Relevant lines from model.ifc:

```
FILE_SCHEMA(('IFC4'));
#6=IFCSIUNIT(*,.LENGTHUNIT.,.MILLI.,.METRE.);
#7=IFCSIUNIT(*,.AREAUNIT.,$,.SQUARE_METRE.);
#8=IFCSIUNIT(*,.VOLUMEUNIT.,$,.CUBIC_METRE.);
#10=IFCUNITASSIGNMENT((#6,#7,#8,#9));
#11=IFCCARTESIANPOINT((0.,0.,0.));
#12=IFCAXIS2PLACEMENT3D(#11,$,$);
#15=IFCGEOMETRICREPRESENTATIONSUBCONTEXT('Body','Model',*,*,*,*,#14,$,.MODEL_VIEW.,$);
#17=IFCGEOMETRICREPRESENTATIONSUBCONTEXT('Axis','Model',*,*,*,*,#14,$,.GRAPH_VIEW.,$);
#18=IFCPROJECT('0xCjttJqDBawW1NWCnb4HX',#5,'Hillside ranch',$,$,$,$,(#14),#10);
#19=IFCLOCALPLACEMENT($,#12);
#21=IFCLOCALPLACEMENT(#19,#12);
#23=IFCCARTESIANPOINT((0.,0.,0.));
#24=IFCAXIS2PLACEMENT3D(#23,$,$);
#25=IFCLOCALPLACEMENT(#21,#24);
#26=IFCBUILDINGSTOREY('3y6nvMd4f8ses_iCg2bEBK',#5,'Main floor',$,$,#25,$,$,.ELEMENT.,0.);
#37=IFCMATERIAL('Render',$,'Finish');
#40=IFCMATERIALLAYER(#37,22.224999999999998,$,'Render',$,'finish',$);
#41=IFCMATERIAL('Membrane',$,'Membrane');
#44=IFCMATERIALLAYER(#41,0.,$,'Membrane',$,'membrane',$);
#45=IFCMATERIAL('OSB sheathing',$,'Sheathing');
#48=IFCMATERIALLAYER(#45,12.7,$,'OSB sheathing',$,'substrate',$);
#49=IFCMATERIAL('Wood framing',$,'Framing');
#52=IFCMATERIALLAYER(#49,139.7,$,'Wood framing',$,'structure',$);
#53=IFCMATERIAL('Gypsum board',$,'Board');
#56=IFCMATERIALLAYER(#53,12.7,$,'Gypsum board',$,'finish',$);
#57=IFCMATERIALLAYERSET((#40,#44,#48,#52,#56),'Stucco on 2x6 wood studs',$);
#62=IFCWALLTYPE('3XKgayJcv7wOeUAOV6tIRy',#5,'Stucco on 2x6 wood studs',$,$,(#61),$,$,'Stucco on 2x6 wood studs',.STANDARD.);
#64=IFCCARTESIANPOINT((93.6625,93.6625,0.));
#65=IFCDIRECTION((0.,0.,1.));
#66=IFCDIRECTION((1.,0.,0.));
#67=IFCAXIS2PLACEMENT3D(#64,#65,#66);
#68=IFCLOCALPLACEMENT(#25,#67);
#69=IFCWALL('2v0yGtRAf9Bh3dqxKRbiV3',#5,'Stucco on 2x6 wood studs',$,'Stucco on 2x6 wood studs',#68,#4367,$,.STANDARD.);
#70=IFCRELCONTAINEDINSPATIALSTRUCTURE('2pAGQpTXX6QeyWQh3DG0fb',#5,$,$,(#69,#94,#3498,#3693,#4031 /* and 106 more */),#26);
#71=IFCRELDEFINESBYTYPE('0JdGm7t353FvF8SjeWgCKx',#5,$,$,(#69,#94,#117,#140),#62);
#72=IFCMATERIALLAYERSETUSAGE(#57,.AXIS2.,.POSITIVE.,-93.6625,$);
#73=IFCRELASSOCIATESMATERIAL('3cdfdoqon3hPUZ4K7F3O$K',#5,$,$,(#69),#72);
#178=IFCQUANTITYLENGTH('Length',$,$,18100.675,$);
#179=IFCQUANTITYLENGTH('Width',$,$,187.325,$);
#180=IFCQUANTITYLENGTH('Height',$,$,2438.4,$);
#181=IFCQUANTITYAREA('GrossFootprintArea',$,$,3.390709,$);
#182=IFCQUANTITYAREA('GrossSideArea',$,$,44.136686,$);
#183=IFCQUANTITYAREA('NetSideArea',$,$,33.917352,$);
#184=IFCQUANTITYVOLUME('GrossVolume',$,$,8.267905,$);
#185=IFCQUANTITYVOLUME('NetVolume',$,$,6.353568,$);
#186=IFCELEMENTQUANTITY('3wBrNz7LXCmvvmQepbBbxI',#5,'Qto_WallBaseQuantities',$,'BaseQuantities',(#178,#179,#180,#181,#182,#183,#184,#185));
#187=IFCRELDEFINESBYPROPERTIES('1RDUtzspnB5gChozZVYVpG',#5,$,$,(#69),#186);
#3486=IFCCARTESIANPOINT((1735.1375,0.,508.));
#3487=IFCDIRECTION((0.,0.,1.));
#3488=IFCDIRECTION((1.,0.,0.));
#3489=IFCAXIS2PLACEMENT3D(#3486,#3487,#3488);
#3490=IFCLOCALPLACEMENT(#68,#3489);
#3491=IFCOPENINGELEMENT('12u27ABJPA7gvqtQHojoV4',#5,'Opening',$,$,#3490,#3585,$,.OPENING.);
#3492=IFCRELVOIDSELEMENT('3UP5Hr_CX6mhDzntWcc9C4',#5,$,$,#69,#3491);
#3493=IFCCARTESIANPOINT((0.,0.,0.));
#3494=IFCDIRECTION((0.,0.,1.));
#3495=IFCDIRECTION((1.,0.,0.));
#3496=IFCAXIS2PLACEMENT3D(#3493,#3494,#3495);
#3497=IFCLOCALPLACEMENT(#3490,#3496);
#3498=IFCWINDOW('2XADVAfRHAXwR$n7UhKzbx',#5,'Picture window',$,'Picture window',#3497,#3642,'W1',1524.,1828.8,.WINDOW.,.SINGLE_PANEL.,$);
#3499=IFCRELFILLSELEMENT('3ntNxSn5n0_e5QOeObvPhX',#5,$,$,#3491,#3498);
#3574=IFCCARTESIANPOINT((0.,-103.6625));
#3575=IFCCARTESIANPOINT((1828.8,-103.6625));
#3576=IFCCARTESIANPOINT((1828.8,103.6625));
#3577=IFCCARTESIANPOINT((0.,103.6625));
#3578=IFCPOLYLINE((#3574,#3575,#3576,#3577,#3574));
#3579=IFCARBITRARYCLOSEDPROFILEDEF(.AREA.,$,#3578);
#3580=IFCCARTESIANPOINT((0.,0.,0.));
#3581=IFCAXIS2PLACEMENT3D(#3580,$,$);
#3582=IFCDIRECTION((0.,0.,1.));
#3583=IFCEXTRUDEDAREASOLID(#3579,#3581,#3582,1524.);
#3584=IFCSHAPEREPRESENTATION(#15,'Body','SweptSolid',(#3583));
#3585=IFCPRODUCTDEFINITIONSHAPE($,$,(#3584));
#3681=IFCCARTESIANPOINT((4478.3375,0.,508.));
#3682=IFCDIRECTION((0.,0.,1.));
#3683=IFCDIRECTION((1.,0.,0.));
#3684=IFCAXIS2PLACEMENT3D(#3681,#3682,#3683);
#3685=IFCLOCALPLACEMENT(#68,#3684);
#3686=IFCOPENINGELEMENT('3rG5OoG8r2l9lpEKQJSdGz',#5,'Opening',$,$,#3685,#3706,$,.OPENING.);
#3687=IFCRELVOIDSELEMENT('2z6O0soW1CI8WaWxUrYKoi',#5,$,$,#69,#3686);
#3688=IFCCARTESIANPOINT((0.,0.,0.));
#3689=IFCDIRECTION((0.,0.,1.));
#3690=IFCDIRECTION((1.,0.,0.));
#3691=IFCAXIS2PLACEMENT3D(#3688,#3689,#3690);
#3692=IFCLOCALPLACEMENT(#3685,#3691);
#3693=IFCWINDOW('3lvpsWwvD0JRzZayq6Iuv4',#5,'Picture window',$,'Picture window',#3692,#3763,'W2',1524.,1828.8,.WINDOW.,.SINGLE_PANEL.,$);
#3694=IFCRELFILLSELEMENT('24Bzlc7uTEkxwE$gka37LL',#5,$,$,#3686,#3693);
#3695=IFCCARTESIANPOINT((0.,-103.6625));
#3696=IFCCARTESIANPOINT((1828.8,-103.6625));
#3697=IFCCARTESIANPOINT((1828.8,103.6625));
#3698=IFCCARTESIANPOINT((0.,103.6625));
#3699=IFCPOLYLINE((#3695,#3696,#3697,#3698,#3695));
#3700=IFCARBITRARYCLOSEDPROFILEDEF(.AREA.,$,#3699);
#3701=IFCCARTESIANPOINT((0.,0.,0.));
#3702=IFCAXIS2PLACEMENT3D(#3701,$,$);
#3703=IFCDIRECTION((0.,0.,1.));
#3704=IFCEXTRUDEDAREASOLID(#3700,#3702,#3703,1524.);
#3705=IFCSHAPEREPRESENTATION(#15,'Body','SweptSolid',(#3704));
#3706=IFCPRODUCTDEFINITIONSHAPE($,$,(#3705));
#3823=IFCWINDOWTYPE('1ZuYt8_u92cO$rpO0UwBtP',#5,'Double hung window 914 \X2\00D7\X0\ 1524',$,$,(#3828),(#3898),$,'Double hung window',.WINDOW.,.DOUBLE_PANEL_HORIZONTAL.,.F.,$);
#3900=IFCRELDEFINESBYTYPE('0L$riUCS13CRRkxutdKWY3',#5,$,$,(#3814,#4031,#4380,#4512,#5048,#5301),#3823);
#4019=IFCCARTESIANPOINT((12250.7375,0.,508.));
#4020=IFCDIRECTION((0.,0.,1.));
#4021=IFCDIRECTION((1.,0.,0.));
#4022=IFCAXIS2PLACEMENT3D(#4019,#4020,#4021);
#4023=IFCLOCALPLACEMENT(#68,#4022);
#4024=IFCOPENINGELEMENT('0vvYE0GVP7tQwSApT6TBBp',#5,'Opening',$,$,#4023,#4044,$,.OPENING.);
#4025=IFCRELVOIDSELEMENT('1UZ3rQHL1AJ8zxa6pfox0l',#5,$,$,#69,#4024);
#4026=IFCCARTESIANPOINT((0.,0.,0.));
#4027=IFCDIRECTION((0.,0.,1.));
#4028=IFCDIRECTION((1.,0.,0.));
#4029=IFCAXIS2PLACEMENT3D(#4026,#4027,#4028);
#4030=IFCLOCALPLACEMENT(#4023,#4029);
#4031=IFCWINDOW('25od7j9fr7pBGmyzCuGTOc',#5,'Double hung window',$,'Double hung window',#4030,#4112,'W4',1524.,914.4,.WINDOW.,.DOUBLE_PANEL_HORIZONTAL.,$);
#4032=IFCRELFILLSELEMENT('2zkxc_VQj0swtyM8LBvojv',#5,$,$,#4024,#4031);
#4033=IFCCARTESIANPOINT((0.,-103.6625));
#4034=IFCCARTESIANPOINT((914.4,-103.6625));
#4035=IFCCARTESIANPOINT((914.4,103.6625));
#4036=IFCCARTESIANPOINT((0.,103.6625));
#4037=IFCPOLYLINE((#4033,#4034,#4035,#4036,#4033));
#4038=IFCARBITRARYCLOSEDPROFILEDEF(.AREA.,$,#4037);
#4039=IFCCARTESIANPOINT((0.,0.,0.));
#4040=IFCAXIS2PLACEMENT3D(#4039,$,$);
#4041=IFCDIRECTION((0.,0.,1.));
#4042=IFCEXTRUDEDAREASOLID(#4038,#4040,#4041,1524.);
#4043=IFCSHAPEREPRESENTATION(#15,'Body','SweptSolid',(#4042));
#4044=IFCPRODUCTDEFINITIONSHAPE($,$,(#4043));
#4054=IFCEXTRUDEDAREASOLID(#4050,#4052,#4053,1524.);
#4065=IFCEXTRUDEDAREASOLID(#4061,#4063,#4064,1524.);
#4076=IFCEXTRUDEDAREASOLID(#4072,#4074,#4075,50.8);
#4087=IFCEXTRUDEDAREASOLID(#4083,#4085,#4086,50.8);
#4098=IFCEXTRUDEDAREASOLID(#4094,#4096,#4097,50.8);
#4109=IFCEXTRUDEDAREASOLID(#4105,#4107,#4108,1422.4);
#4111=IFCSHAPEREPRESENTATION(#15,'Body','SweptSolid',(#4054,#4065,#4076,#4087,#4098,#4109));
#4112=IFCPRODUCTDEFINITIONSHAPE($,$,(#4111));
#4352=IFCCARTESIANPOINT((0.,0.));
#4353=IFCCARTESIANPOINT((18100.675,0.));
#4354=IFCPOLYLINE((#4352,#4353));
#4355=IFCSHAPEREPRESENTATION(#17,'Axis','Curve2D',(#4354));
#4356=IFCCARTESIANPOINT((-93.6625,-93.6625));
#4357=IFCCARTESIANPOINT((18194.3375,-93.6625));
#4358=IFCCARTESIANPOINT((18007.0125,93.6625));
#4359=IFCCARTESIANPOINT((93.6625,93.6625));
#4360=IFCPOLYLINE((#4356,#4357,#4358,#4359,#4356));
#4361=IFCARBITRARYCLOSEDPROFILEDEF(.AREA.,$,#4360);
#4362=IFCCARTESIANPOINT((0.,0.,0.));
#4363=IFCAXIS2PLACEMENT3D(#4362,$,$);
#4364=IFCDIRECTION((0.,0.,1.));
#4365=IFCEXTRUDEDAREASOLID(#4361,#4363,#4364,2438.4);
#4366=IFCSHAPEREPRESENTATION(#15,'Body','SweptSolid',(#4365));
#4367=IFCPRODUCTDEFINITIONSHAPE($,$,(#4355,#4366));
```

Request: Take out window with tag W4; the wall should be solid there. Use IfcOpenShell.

```python
import ifcopenshell
import ifcopenshell.api.feature
import ifcopenshell.api.pset
import ifcopenshell.api.root
import ifcopenshell.geom
import ifcopenshell.util.element
import ifcopenshell.util.shape
import ifcopenshell.util.unit

model = ifcopenshell.open("model.ifc")
area_scale = ifcopenshell.util.unit.calculate_unit_scale(model, "AREAUNIT")
volume_scale = ifcopenshell.util.unit.calculate_unit_scale(model, "VOLUMEUNIT")
settings = ifcopenshell.geom.settings()


def volume(element):
    """Net volume in cubic metres, openings subtracted."""
    shape = ifcopenshell.geom.create_shape(settings, element)
    return ifcopenshell.util.shape.get_volume(shape.geometry)


window = model.by_id(4031)
opening = window.FillsVoids[0].RelatingOpeningElement
wall = opening.VoidsElements[0].RelatingBuildingElement
before = volume(wall)

ifcopenshell.api.root.remove_product(model, product=window)
ifcopenshell.api.feature.remove_feature(model, feature=opening)

after = volume(wall)
thickness = 0.1873  # wall thickness in metres

# Update the wall's stored quantities.
qto = model.by_id(ifcopenshell.util.element.get_pset(wall, "Qto_WallBaseQuantities", should_inherit=False)["id"])
ifcopenshell.api.pset.edit_qto(model, qto=qto, properties={
    "NetSideArea": after / thickness / area_scale,
    "NetVolume": after / volume_scale,
})

print(f"wall volume {before:.3f} -> {after:.3f} m3")

model.write("model_updated.ifc")
```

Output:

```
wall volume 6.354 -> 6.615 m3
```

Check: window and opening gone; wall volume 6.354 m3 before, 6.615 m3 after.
